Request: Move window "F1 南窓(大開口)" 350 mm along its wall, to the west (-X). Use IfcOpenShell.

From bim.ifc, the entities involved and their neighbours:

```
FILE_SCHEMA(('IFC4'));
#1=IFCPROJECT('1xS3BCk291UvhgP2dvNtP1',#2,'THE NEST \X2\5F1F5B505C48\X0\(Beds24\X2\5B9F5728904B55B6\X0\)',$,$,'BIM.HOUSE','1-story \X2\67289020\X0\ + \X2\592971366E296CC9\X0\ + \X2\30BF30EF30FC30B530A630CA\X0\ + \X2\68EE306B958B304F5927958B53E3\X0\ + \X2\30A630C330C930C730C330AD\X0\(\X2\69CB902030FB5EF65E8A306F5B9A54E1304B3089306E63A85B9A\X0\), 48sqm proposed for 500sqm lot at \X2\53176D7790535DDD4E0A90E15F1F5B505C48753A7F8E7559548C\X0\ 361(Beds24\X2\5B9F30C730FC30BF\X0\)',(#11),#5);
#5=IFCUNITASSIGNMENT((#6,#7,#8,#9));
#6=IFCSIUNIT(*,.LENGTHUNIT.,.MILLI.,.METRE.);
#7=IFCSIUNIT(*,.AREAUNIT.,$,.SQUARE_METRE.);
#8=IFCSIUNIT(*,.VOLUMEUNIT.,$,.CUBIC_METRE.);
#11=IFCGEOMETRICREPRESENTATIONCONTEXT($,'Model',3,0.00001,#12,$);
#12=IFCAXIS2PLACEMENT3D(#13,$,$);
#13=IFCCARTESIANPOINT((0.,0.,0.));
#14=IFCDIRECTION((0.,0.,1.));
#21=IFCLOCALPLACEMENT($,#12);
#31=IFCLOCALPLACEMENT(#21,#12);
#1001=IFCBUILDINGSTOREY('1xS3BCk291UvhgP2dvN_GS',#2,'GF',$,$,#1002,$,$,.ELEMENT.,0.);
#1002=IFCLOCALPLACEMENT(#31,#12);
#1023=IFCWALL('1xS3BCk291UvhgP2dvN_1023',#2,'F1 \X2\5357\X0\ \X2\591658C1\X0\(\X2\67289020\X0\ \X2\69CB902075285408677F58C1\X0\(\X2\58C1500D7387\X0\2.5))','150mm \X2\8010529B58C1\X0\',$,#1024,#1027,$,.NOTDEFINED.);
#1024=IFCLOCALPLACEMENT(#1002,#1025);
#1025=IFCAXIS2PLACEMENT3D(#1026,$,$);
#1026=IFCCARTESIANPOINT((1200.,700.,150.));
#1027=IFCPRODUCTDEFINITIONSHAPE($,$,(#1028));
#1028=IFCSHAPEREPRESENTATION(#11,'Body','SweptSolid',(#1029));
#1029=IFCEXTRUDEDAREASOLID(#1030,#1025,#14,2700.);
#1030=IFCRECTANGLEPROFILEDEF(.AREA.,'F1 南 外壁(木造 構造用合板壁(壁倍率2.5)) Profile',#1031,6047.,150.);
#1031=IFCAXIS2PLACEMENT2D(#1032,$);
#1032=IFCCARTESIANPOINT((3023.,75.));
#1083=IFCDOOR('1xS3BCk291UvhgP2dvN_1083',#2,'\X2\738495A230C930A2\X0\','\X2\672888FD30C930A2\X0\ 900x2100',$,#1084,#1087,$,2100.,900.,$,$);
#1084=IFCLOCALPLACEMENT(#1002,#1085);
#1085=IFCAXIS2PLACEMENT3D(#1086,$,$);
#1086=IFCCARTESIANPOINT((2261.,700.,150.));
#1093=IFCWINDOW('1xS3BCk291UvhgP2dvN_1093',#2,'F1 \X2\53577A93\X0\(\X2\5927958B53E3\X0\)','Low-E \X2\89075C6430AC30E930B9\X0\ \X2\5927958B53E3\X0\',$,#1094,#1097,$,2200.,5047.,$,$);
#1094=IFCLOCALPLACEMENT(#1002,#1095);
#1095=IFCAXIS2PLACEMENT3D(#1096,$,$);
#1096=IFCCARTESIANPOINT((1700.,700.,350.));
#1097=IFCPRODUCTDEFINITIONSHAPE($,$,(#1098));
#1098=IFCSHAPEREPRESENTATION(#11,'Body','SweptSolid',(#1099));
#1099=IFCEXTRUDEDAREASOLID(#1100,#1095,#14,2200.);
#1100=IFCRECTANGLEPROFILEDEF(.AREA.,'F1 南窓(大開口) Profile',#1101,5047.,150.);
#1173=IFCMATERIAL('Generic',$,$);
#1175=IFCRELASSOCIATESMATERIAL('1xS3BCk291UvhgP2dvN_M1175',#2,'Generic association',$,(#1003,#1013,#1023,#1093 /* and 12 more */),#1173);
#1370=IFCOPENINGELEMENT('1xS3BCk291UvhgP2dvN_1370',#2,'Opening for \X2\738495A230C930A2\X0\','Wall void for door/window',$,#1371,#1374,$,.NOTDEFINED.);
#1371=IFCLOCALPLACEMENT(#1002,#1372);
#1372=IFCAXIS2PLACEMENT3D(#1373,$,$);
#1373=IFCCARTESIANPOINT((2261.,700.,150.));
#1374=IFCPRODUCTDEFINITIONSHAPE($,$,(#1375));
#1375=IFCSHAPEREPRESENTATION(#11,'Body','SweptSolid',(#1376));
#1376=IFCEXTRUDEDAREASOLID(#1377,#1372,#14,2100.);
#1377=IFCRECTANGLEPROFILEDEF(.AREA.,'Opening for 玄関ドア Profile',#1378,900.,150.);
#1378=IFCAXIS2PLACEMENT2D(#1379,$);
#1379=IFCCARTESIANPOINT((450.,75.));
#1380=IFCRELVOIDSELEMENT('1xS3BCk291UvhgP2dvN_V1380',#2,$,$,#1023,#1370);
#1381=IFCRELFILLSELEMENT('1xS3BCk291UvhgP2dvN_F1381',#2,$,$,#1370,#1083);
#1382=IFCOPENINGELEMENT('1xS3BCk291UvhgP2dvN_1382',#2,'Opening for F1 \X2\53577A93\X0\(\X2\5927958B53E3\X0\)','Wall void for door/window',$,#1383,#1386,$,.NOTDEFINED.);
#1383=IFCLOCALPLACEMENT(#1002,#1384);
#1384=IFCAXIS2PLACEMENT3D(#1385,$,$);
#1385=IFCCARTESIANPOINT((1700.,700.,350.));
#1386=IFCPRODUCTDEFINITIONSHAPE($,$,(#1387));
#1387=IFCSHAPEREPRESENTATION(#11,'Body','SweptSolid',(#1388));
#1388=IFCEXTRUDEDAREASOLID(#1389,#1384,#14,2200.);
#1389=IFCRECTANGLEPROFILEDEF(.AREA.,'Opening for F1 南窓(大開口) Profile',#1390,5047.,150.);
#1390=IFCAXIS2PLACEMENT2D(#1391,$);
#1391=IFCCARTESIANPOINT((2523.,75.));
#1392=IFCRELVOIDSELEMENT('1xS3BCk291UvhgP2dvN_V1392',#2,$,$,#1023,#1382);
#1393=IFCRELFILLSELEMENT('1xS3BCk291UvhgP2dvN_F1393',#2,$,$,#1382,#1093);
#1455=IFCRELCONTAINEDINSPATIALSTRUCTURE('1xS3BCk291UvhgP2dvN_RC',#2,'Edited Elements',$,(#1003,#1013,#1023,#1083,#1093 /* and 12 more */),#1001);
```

```python
import ifcopenshell
import ifcopenshell.api.geometry
import ifcopenshell.util.placement

model = ifcopenshell.open("bim.ifc")

window = model.by_guid("1xS3BCk291UvhgP2dvN_1093")
opening = window.FillsVoids[0].RelatingOpeningElement
wall = opening.VoidsElements[0].RelatingBuildingElement

wall_matrix = ifcopenshell.util.placement.get_local_placement(wall.ObjectPlacement)
shift = wall_matrix[:3, 0] * -350.0
before = ifcopenshell.util.placement.get_local_placement(window.ObjectPlacement)[:3, 3].copy()

# The window is not placed relative to its opening, so move both.
for product in (opening, window):
    matrix = ifcopenshell.util.placement.get_local_placement(product.ObjectPlacement)
    matrix[:3, 3] += shift
    ifcopenshell.api.geometry.edit_object_placement(model, product=product, matrix=matrix, is_si=False)

after = ifcopenshell.util.placement.get_local_placement(window.ObjectPlacement)[:3, 3]
print("window moved by", (after - before).round(3) + 0.0)

model.write("bim_updated.ifc")
```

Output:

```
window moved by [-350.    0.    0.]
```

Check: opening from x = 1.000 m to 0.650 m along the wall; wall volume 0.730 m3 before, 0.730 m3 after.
